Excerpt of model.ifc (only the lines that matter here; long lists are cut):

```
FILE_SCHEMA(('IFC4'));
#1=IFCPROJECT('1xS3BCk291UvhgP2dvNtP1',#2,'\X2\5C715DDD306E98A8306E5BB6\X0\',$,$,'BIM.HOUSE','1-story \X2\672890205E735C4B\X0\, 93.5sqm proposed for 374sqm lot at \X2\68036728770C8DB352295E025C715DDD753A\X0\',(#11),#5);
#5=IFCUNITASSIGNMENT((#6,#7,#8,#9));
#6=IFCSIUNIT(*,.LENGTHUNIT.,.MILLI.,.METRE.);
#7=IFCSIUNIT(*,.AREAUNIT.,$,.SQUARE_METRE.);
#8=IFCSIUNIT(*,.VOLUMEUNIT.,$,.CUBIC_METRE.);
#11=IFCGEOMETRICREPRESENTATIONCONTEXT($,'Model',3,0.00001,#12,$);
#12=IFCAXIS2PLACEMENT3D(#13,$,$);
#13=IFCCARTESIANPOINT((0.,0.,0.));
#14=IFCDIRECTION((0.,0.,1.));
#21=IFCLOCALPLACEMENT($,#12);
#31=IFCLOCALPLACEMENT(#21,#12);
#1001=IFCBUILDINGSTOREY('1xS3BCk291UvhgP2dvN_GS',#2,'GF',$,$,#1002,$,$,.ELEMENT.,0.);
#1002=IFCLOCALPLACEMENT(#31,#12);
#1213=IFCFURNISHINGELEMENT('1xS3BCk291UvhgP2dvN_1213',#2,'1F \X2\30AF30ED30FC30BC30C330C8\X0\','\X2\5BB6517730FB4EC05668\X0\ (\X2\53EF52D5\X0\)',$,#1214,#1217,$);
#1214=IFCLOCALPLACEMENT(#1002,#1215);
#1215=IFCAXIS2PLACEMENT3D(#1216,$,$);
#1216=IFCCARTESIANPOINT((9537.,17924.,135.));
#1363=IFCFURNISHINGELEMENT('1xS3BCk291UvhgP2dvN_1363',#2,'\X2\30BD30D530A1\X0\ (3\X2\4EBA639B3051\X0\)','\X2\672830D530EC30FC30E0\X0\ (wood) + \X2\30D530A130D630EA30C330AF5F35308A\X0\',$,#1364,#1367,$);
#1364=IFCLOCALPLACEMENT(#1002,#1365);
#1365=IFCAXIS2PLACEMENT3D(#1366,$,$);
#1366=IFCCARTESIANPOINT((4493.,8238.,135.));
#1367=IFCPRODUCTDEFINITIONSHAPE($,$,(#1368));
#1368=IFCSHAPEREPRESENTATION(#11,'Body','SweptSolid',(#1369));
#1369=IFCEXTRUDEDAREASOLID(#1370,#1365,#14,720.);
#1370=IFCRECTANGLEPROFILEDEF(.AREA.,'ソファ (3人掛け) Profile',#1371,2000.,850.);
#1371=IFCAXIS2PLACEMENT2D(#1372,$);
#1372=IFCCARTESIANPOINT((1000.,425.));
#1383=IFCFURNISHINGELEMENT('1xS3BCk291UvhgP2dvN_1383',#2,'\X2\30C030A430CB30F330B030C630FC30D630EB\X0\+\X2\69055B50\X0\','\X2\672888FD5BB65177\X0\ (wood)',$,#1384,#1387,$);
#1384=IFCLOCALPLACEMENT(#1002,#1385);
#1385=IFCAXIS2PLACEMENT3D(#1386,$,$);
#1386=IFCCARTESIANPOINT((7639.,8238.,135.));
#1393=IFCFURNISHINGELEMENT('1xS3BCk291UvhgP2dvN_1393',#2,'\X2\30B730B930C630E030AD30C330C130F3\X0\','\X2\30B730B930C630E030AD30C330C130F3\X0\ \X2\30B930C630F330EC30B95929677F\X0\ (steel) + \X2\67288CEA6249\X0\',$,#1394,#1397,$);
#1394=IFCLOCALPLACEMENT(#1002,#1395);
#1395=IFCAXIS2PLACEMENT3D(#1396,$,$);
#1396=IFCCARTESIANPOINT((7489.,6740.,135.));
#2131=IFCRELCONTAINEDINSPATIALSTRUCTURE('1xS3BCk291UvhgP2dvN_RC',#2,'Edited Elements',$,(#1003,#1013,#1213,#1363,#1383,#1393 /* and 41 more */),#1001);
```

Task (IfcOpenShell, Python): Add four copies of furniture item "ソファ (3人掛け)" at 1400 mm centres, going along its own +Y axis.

```python
import ifcopenshell
import ifcopenshell.api.geometry
import ifcopenshell.api.root
import ifcopenshell.util.element
import ifcopenshell.util.placement
import ifcopenshell.util.unit

model = ifcopenshell.open("model.ifc")
unit_scale = ifcopenshell.util.unit.calculate_unit_scale(model)


def reuse_history(source, copy):
    """copy_class also copies each property set's owner history, people and application; keep the originals."""
    for rel in copy.IsDefinedBy:
        if rel.is_a("IfcRelDefinesByProperties") and (history := rel.RelatingPropertyDefinition.OwnerHistory):
            rel.RelatingPropertyDefinition.OwnerHistory = source.OwnerHistory
            ifcopenshell.util.element.remove_deep2(model, history)


source = model.by_guid("1xS3BCk291UvhgP2dvN_1363")
base = ifcopenshell.util.placement.get_local_placement(source.ObjectPlacement)
step = base[:3, 1] * 1.4 / unit_scale

for i in range(1, 5):
    copy = ifcopenshell.api.root.copy_class(model, product=source)
    copy.Representation = ifcopenshell.util.element.copy_deep(
        model, source.Representation, exclude=["IfcGeometricRepresentationContext", "IfcRepresentationMap"]
    )
    reuse_history(source, copy)
    matrix = base.copy()
    matrix[:3, 3] += i * step
    print("added at", matrix[:3, 3].round(3) + 0.0)
    ifcopenshell.api.geometry.edit_object_placement(model, product=copy, matrix=matrix, is_si=False)

model.write("model_edited.ifc")
```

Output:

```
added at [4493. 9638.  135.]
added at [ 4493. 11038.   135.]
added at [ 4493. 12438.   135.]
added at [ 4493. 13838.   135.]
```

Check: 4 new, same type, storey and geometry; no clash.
